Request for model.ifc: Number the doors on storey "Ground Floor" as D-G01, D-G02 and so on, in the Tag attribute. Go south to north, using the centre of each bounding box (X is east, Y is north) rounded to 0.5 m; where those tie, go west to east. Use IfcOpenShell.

First a look at what the model holds.

```python
import ifcopenshell
import ifcopenshell.util.element
import ifcopenshell.util.placement

model = ifcopenshell.open("model.ifc")
print(model.schema)
storey = next(s for s in model.by_type("IfcBuildingStorey") if s.Name == "Ground Floor")
doors = [e for e in ifcopenshell.util.element.get_decomposition(storey) if e.is_a("IfcDoor")]
for e in sorted(doors, key=lambda e: e.id()):
    origin = ifcopenshell.util.placement.get_local_placement(e.ObjectPlacement)[:3, 3]
    print(e.id(), e.Tag, e.Name, origin.round(2) + 0.0, sep=" | ")
```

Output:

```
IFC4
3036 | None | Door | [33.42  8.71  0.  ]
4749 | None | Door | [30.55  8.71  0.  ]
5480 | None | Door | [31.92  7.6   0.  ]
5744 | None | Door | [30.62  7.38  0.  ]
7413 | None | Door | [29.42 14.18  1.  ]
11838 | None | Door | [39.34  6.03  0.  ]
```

```python
import ifcopenshell
import ifcopenshell.geom
import ifcopenshell.util.element
import ifcopenshell.util.shape

model = ifcopenshell.open("model.ifc")
settings = ifcopenshell.geom.settings()
settings.set("use-world-coords", True)


def centre(element):
    shape = ifcopenshell.geom.create_shape(settings, element)
    return ifcopenshell.util.shape.get_bbox_centroid(shape.geometry)


storey = next(s for s in model.by_type("IfcBuildingStorey") if s.Name == "Ground Floor")
doors = [e for e in ifcopenshell.util.element.get_decomposition(storey) if e.is_a("IfcDoor")]

# Insertion points can sit at a corner or the storey origin, so sort by the geometry (in metres).
centres = {e: centre(e) for e in doors}
doors.sort(key=lambda e: (round(centres[e][1] / 0.5), centres[e][0]))

for i, e in enumerate(doors, start=1):
    number = f"D-G{i:02d}"
    e.Tag = number
    print(e.id(), number)

model.write("model_rev.ifc")
```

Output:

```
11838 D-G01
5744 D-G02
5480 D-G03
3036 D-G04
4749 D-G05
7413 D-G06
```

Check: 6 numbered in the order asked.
